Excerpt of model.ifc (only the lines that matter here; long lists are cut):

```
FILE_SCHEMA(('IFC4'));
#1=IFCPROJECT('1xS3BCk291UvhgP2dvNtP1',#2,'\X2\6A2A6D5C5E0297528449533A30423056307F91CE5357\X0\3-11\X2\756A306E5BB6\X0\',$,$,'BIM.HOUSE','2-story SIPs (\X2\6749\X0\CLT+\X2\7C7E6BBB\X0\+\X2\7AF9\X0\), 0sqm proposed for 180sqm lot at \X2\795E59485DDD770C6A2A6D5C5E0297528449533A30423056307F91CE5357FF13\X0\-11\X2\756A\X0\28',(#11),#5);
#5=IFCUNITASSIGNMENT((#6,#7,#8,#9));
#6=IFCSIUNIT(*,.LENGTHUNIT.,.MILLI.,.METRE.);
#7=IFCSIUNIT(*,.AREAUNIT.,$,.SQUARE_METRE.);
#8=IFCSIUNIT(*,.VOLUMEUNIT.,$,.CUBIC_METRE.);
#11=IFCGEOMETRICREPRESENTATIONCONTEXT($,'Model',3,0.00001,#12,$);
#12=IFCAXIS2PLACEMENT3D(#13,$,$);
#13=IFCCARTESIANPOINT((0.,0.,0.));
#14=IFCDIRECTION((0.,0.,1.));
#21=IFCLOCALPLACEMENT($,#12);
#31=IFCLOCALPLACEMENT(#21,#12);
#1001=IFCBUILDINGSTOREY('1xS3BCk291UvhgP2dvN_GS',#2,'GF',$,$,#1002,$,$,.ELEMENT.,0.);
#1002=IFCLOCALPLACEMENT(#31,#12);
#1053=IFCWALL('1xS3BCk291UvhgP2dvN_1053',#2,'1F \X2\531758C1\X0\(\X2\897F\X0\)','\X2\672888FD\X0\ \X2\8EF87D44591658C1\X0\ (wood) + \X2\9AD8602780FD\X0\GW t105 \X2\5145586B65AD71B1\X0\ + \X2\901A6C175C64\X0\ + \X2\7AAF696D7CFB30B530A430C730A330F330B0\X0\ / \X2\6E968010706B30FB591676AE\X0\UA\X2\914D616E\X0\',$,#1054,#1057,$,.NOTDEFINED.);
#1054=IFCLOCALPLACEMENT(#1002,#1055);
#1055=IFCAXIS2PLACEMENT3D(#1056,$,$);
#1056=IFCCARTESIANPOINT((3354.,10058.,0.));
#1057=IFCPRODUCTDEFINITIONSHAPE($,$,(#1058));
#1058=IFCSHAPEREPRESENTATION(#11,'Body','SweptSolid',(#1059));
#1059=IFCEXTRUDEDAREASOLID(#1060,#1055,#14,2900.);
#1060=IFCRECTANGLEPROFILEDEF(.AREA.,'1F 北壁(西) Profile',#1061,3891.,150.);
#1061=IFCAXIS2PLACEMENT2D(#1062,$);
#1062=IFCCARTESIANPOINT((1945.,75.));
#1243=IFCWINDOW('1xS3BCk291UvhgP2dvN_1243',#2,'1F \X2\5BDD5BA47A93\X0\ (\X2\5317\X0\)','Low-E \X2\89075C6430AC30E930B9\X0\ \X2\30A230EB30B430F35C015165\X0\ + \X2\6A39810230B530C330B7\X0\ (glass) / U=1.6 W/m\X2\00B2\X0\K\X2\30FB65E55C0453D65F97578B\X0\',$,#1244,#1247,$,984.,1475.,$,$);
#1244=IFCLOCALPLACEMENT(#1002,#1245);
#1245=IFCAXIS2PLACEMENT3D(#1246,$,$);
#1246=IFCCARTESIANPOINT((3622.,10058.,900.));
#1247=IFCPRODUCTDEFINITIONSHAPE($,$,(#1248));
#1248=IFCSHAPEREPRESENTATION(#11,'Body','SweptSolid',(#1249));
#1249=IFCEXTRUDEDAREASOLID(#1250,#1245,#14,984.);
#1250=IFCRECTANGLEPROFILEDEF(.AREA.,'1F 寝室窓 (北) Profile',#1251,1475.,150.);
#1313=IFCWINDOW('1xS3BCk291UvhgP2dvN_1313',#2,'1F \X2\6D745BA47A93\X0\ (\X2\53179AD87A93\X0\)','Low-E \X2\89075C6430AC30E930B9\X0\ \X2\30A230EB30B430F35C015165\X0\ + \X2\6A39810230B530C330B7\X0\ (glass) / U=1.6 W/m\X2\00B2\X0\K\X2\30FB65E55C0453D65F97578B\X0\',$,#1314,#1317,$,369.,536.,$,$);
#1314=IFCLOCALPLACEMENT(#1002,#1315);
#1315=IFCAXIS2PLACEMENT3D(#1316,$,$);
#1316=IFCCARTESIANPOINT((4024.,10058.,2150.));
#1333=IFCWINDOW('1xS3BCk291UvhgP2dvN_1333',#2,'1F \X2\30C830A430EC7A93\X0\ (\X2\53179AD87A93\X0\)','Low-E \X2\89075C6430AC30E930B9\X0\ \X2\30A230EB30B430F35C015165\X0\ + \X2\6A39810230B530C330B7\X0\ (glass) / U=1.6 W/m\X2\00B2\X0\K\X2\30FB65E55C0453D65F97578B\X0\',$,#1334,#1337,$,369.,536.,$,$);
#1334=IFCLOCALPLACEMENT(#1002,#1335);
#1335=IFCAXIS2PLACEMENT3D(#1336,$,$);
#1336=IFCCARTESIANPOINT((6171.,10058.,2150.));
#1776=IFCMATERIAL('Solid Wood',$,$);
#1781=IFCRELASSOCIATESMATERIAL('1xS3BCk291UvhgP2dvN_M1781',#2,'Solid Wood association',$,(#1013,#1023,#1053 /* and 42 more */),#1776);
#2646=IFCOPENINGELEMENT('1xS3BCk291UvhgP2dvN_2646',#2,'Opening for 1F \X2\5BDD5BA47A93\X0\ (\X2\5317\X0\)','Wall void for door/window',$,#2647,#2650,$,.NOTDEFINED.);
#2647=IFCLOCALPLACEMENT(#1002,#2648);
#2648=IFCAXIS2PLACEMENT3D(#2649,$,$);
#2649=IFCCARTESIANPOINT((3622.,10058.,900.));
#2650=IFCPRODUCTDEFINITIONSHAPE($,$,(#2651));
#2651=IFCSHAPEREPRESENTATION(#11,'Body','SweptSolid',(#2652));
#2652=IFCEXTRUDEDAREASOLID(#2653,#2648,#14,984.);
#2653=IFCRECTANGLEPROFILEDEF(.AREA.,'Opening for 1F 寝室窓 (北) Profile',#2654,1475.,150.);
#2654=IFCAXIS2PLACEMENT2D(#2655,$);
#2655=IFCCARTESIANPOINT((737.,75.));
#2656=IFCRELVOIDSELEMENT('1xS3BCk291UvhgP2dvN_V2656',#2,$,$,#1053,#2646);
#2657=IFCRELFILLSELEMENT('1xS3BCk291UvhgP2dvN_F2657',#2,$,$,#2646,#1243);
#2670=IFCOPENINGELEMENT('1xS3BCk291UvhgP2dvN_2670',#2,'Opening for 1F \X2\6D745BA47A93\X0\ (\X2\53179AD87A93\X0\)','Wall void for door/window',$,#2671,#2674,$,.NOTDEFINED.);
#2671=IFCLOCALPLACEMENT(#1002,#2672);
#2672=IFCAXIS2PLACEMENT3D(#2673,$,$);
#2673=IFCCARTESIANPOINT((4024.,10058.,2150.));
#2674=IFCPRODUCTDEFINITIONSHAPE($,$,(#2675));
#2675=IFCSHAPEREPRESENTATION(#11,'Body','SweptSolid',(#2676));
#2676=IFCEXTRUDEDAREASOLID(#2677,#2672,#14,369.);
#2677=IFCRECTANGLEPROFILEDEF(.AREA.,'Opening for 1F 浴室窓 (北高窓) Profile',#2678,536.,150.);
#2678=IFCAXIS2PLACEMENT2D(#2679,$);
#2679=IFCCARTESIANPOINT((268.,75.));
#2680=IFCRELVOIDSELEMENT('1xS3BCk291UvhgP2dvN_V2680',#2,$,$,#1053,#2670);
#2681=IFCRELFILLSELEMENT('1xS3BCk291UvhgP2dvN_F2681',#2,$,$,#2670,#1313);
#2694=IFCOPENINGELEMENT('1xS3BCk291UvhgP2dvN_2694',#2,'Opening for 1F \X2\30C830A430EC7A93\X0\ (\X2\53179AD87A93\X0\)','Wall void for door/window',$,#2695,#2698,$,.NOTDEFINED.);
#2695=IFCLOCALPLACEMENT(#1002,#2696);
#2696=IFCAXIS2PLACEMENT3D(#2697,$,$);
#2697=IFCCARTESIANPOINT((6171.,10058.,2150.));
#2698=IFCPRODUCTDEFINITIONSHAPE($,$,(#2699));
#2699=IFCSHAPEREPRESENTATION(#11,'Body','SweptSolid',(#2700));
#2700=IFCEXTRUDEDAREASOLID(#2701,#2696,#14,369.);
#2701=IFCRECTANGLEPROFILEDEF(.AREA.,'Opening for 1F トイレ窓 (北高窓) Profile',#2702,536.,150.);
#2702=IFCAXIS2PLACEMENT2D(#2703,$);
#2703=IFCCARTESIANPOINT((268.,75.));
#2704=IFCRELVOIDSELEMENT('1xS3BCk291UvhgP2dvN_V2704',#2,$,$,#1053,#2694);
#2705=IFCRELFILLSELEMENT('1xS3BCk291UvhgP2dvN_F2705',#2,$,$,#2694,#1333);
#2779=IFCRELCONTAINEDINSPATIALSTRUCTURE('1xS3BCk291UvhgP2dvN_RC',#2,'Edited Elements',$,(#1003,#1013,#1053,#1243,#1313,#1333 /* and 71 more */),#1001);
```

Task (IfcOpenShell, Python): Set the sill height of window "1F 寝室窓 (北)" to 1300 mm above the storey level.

```python
import numpy as np
import ifcopenshell
import ifcopenshell.api.geometry
import ifcopenshell.geom
import ifcopenshell.util.element
import ifcopenshell.util.placement
import ifcopenshell.util.shape
import ifcopenshell.util.unit

model = ifcopenshell.open("model.ifc")
unit_scale = ifcopenshell.util.unit.calculate_unit_scale(model)

window = model.by_guid("1xS3BCk291UvhgP2dvN_1243")
opening = window.FillsVoids[0].RelatingOpeningElement
storey = ifcopenshell.util.element.get_container(window, ifc_class="IfcBuildingStorey")
level = ifcopenshell.util.placement.get_local_placement(storey.ObjectPlacement)[2, 3]

# The opening's origin need not be at the sill, so measure its lowest point.
shape = ifcopenshell.geom.create_shape(ifcopenshell.geom.settings(), opening)
bottom = ifcopenshell.util.shape.get_shape_bottom_elevation(shape, shape.geometry) / unit_scale
dz = level + 1300.0 - bottom

shift = np.array([0.0, 0.0, dz])
# The window is not placed relative to its opening, so move both.
for product in (opening, window):
    matrix = ifcopenshell.util.placement.get_local_placement(product.ObjectPlacement)
    matrix[:3, 3] += shift
    ifcopenshell.api.geometry.edit_object_placement(model, product=product, matrix=matrix, is_si=False)

print(f"moved by {dz * unit_scale:+.3f} m")

model.write("model_rev.ifc")
```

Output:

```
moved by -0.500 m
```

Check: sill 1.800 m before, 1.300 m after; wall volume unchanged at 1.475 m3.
